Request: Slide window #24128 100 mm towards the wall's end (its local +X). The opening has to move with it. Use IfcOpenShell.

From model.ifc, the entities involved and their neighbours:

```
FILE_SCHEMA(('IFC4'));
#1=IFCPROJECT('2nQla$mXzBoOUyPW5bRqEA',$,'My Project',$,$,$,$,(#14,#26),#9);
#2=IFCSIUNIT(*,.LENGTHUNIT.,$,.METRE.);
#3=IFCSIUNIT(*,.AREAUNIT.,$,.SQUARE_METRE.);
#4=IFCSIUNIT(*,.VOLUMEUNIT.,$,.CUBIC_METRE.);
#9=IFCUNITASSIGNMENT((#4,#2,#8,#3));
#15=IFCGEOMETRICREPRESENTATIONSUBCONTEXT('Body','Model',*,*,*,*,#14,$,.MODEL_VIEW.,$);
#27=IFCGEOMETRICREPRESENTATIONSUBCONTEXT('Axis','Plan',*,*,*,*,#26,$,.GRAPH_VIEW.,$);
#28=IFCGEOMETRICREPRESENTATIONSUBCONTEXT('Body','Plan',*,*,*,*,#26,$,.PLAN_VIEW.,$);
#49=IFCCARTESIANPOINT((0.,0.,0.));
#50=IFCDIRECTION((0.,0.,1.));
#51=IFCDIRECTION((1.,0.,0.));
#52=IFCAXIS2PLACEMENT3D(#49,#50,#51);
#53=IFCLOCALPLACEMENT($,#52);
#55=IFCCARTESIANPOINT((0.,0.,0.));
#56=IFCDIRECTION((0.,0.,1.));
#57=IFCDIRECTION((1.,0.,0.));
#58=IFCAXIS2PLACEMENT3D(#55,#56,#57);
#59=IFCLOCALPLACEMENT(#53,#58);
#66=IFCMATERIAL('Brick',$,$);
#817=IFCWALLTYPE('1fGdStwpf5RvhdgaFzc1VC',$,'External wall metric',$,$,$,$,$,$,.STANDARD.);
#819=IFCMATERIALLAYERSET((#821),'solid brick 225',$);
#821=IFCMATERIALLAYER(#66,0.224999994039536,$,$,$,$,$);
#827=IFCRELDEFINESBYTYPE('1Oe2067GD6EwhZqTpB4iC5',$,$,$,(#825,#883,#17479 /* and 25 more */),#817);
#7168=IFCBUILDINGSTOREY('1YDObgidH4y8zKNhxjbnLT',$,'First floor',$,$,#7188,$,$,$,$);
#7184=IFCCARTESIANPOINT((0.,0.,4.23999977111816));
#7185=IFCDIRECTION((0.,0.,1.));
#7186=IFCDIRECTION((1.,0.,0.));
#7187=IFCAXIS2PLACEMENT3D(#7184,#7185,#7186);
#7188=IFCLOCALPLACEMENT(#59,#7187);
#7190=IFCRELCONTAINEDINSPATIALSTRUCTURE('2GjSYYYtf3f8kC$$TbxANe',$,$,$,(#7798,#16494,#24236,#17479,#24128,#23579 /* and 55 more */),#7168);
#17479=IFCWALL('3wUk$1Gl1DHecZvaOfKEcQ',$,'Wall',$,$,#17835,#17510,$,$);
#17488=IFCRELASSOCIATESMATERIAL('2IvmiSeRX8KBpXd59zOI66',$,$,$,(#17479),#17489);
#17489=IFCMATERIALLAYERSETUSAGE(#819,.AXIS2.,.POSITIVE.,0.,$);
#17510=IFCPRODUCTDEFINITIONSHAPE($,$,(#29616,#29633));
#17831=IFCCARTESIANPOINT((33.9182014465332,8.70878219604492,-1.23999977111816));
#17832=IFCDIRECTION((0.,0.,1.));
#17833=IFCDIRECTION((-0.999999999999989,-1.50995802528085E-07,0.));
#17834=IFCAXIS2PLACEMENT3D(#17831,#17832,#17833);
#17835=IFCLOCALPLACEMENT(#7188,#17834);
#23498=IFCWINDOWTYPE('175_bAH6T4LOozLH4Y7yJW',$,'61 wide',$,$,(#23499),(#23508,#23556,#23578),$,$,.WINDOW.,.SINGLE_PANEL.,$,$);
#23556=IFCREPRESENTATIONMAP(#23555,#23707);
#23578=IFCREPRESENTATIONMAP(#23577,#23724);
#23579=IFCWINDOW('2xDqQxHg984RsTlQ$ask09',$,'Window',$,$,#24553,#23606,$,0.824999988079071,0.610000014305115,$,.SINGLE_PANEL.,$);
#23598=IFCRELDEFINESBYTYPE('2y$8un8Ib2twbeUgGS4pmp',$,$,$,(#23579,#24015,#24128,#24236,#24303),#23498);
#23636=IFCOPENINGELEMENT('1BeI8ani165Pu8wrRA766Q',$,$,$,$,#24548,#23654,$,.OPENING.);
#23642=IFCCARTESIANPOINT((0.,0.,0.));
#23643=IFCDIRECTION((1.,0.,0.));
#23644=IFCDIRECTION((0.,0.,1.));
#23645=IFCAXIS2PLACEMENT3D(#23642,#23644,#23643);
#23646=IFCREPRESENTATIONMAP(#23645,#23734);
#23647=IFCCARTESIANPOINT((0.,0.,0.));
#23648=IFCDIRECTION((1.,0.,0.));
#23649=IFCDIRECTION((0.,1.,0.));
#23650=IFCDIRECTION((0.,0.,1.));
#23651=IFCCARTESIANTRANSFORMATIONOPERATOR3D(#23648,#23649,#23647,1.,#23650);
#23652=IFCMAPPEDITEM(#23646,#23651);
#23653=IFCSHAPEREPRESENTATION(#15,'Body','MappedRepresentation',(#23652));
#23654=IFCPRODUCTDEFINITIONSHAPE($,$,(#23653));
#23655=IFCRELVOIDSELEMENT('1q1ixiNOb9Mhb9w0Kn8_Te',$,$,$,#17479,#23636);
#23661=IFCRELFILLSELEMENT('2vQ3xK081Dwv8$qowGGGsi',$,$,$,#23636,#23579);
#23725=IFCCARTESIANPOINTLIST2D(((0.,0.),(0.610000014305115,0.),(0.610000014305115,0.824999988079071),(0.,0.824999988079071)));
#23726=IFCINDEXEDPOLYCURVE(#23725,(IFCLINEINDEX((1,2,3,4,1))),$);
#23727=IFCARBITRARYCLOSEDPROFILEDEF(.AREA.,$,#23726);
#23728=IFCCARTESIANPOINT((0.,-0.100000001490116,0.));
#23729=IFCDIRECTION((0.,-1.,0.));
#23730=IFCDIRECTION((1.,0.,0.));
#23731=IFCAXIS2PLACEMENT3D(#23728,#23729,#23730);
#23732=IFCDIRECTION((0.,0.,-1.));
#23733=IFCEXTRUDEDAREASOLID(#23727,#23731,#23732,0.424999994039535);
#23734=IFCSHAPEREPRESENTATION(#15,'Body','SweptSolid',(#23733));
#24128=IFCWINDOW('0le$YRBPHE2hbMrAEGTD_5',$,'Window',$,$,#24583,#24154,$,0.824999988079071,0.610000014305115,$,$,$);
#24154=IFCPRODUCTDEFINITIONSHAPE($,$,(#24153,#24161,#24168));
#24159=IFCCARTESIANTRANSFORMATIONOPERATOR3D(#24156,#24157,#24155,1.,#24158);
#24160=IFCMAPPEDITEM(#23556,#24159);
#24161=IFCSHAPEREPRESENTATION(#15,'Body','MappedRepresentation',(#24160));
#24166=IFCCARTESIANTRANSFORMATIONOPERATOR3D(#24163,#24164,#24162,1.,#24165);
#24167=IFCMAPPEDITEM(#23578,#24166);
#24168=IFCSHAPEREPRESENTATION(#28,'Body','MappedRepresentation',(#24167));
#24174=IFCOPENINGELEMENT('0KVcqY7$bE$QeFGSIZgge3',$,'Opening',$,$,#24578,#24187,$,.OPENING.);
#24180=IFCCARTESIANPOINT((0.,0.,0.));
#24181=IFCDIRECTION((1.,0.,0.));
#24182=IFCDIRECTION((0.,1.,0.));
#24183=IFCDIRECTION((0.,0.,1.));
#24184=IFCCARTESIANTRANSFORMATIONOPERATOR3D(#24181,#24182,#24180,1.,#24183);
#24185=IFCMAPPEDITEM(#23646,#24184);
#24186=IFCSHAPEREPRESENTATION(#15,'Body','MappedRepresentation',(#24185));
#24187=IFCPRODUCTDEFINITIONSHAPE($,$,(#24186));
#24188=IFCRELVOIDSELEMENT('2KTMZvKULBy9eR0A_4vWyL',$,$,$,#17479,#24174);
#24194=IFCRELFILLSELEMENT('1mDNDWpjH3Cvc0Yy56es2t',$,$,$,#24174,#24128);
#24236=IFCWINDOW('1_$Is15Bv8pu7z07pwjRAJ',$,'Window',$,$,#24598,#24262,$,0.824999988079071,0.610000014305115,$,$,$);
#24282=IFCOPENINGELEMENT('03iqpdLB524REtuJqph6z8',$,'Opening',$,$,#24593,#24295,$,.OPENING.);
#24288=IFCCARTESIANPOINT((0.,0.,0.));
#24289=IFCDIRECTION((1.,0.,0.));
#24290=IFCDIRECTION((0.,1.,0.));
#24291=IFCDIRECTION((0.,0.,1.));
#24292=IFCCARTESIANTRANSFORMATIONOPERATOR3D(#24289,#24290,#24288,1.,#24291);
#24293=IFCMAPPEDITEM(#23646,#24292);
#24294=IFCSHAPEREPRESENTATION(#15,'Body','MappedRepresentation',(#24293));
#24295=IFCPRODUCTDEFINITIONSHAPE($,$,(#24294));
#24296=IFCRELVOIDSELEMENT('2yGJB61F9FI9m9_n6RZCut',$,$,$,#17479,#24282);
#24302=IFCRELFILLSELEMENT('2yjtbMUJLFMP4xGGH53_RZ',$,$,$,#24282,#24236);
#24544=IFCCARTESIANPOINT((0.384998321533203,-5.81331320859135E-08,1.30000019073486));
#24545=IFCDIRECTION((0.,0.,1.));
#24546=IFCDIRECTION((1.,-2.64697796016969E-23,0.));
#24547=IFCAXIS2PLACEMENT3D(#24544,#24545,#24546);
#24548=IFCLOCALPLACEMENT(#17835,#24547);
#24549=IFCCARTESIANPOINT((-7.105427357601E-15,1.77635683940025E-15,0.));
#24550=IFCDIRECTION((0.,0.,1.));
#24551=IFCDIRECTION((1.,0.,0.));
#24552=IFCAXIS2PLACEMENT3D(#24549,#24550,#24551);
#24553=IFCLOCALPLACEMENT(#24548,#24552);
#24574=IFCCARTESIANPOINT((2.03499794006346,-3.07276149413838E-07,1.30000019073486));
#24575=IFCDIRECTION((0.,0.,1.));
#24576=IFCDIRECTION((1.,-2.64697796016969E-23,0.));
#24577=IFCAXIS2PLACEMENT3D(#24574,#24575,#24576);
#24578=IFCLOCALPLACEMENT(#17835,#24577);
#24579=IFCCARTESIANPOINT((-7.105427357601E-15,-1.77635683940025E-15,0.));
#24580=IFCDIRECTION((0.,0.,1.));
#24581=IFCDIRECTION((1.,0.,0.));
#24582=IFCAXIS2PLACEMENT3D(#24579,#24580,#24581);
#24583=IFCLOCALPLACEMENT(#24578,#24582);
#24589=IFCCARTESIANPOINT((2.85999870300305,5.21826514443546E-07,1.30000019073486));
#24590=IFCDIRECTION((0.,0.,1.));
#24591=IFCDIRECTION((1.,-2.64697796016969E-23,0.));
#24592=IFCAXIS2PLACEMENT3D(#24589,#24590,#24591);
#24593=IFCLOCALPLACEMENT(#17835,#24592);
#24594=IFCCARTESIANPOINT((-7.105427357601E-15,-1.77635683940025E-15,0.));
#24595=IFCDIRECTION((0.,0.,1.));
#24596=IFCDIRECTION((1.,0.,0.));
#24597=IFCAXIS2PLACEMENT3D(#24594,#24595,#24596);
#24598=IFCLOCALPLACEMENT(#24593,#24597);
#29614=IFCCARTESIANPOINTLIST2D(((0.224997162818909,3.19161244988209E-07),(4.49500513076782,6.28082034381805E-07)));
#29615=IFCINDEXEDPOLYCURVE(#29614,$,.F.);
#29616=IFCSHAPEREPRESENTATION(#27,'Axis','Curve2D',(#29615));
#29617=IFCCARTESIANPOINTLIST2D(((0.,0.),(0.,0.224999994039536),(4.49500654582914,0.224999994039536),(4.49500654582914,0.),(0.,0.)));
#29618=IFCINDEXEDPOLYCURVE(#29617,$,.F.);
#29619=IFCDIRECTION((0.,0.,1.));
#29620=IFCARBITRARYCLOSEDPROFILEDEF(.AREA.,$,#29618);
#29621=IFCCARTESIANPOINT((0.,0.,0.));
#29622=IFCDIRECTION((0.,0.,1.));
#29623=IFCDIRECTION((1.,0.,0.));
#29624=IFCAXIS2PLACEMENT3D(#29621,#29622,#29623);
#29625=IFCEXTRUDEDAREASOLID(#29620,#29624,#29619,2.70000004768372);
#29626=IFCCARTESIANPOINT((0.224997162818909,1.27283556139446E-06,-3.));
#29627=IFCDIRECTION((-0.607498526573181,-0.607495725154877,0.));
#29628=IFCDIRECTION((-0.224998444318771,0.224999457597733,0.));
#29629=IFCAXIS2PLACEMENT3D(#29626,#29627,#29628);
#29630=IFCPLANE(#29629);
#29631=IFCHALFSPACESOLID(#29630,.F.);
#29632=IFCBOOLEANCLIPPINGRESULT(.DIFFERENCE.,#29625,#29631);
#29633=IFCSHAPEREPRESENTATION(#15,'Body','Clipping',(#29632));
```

```python
import ifcopenshell
import ifcopenshell.api.geometry
import ifcopenshell.util.placement
import ifcopenshell.util.unit

model = ifcopenshell.open("model.ifc")
unit_scale = ifcopenshell.util.unit.calculate_unit_scale(model)

window = model.by_guid("0le$YRBPHE2hbMrAEGTD_5")
opening = window.FillsVoids[0].RelatingOpeningElement
wall = opening.VoidsElements[0].RelatingBuildingElement

wall_matrix = ifcopenshell.util.placement.get_local_placement(wall.ObjectPlacement)
shift = wall_matrix[:3, 0] * 0.1 / unit_scale
before = ifcopenshell.util.placement.get_local_placement(window.ObjectPlacement)[:3, 3].copy()

# The window is placed relative to its opening, so it follows when the opening moves.
matrix = ifcopenshell.util.placement.get_local_placement(opening.ObjectPlacement)
matrix[:3, 3] += shift
ifcopenshell.api.geometry.edit_object_placement(
    model, product=opening, matrix=matrix, is_si=False, should_transform_children=True
)

after = ifcopenshell.util.placement.get_local_placement(window.ObjectPlacement)[:3, 3]
print("window moved by", (after - before).round(3) + 0.0)

model.write("model_updated.ifc")
```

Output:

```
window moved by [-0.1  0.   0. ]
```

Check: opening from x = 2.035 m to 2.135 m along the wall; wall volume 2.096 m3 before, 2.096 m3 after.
